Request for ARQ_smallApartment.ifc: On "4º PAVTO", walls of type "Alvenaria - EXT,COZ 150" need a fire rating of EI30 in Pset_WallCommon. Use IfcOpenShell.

First a look at what the model holds.

```python
import ifcopenshell
import ifcopenshell.util.element

model = ifcopenshell.open("ARQ_smallApartment.ifc")
print(model.schema)
storey = next(s for s in model.by_type("IfcBuildingStorey") if s.Name == "4º PAVTO")
walls = [e for e in ifcopenshell.util.element.get_decomposition(storey) if e.is_a("IfcWall")]
seen = {}
for e in walls:
    element_type = ifcopenshell.util.element.get_type(e)
    key = (element_type.Name if element_type != e and element_type else None, ifcopenshell.util.element.get_pset(e, "Pset_WallCommon", "FireRating"))
    seen[key] = seen.get(key, 0) + 1
for (name, value), count in sorted(seen.items(), key=str):
    print(count, "x", name, "|", value)
```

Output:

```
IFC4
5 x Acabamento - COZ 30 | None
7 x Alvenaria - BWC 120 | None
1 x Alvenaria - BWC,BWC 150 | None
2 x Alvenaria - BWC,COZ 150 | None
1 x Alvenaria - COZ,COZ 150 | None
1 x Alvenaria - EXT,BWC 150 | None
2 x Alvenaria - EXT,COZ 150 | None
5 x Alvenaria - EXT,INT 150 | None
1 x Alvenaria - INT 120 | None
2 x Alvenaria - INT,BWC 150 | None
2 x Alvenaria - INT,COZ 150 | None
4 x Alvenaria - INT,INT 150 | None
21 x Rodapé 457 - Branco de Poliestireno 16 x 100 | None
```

```python
import ifcopenshell
import ifcopenshell.api.pset
import ifcopenshell.util.element

model = ifcopenshell.open("ARQ_smallApartment.ifc")

storey = next(s for s in model.by_type("IfcBuildingStorey") if s.Name == "4º PAVTO")
walls = [e for e in ifcopenshell.util.element.get_decomposition(storey) if e.is_a("IfcWall")]

count = 0
for e in walls:
    element_type = ifcopenshell.util.element.get_type(e)
    if element_type in (None, e) or element_type.Name != "Alvenaria - EXT,COZ 150":
        continue
    # add_pset returns the element's existing set when there is one.
    pset = ifcopenshell.api.pset.add_pset(model, product=e, name="Pset_WallCommon")
    ifcopenshell.api.pset.edit_pset(model, pset=pset, properties={"FireRating": "EI30"})
    count += 1

print(count, "walls updated")

model.write("ARQ_smallApartment_edited.ifc")
```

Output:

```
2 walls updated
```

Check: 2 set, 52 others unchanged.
